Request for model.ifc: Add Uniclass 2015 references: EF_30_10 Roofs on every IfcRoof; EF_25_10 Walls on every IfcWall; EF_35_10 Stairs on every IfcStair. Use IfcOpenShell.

First a look at what the model holds.

```python
import ifcopenshell

model = ifcopenshell.open("model.ifc")
print(model.schema)
print("classifications:", [c.Name for c in model.by_type("IfcClassification")])
for ifc_class in ("IfcDoor", "IfcRoof", "IfcStair", "IfcWall", "IfcWindow"):
    print(ifc_class, len(model.by_type(ifc_class)))
```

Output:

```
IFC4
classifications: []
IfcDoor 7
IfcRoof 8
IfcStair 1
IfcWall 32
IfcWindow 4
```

```python
import ifcopenshell
import ifcopenshell.api.classification

model = ifcopenshell.open("model.ifc")

system = ifcopenshell.api.classification.add_classification(model, classification="Uniclass 2015")

codes = {
    "IfcRoof": ("EF_30_10", "Roofs"),
    "IfcWall": ("EF_25_10", "Walls"),
    "IfcStair": ("EF_35_10", "Stairs"),
}
for ifc_class, (code, name) in codes.items():
    products = model.by_type(ifc_class)
    ifcopenshell.api.classification.add_reference(
        model, products=products, classification=system, identification=code, name=name
    )
    print(code, len(products))

model.write("model_updated.ifc")
```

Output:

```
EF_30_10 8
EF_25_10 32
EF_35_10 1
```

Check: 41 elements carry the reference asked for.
